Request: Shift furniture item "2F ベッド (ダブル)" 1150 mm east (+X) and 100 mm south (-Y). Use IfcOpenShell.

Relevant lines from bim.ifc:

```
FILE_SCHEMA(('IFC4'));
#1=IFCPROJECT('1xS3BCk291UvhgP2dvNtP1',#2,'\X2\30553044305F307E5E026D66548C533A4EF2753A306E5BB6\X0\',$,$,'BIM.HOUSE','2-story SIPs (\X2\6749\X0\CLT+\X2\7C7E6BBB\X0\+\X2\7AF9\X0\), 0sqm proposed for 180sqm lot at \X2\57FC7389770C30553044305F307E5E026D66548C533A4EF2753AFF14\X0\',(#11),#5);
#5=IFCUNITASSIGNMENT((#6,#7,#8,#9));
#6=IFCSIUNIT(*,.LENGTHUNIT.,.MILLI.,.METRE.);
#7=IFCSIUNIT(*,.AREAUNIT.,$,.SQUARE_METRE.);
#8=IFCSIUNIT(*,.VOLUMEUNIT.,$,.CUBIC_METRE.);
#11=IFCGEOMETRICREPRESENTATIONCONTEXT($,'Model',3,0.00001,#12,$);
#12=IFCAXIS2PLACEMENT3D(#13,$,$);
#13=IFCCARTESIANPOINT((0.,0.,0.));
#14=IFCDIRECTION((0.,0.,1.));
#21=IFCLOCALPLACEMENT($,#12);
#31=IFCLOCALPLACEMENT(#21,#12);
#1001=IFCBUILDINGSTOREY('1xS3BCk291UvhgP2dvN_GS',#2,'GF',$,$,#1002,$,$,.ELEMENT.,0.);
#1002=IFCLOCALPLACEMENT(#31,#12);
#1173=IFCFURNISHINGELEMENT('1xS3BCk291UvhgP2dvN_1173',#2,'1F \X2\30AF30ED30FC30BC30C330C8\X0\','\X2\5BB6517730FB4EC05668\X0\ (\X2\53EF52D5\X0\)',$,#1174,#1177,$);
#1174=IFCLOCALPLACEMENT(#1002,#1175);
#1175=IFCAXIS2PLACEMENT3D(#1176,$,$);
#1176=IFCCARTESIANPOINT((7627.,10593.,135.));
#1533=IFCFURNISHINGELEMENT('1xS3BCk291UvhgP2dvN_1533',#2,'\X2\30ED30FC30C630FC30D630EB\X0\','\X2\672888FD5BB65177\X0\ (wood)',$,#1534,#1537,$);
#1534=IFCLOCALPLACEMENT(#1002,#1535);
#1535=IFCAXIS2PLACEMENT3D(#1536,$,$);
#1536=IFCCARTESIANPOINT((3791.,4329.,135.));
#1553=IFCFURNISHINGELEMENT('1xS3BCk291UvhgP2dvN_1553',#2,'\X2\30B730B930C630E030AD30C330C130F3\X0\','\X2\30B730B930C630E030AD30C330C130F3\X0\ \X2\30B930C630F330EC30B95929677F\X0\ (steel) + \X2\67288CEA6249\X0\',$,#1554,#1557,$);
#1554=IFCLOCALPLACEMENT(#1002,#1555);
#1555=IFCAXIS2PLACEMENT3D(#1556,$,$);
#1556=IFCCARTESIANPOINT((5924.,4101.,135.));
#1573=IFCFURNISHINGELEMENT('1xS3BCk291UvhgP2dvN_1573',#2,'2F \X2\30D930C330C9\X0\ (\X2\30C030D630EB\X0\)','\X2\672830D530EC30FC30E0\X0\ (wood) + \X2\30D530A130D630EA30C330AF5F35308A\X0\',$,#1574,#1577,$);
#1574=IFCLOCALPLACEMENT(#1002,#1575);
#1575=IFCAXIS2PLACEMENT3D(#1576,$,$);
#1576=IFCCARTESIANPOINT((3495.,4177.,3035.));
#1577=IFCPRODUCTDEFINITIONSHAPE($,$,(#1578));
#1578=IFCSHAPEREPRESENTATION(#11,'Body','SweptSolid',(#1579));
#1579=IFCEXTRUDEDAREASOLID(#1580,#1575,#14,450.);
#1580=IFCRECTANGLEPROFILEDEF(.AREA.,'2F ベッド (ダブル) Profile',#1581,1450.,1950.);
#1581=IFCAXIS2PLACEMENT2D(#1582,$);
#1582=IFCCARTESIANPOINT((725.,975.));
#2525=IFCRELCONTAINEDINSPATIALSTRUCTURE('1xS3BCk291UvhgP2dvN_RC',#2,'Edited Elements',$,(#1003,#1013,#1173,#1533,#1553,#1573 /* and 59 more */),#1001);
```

```python
import ifcopenshell
import ifcopenshell.api.geometry
import ifcopenshell.util.placement

model = ifcopenshell.open("bim.ifc")

item = model.by_guid("1xS3BCk291UvhgP2dvN_1573")
matrix = ifcopenshell.util.placement.get_local_placement(item.ObjectPlacement)
matrix[0, 3] += 1150.0
matrix[1, 3] -= 100.0
ifcopenshell.api.geometry.edit_object_placement(model, product=item, matrix=matrix, is_si=False)

print(ifcopenshell.util.placement.get_local_placement(item.ObjectPlacement).round(3) + 0.0)

model.write("bim_v2.ifc")
```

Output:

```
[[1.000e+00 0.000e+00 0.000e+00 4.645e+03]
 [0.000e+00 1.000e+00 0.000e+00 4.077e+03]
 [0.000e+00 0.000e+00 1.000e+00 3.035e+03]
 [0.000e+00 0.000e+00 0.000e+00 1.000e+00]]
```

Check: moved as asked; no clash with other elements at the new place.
